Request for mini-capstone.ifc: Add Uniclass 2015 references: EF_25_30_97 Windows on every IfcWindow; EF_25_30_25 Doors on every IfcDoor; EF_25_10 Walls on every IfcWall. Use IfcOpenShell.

First a look at what the model holds.

```python
import ifcopenshell

model = ifcopenshell.open("mini-capstone.ifc")
print(model.schema)
print("classifications:", [c.Name for c in model.by_type("IfcClassification")])
for ifc_class in ("IfcDoor", "IfcRoof", "IfcStair", "IfcWall", "IfcWindow"):
    print(ifc_class, len(model.by_type(ifc_class)))
```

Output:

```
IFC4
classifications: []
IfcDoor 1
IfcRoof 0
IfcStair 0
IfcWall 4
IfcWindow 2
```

```python
import ifcopenshell
import ifcopenshell.api.classification

model = ifcopenshell.open("mini-capstone.ifc")

system = ifcopenshell.api.classification.add_classification(model, classification="Uniclass 2015")

codes = {
    "IfcWindow": ("EF_25_30_97", "Windows"),
    "IfcDoor": ("EF_25_30_25", "Doors"),
    "IfcWall": ("EF_25_10", "Walls"),
}
for ifc_class, (code, name) in codes.items():
    products = model.by_type(ifc_class)
    ifcopenshell.api.classification.add_reference(
        model, products=products, classification=system, identification=code, name=name
    )
    print(code, len(products))

model.write("mini-capstone_v2.ifc")
```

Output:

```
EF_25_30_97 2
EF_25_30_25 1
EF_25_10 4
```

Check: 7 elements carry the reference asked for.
